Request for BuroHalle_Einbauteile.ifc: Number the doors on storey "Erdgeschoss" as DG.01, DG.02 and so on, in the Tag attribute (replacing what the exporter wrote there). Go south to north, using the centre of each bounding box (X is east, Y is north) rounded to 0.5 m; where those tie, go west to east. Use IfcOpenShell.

First a look at what the model holds.

```python
import ifcopenshell
import ifcopenshell.util.element
import ifcopenshell.util.placement

model = ifcopenshell.open("BuroHalle_Einbauteile.ifc")
print(model.schema)
storey = next(s for s in model.by_type("IfcBuildingStorey") if s.Name == "Erdgeschoss")
doors = [e for e in ifcopenshell.util.element.get_decomposition(storey) if e.is_a("IfcDoor")]
for e in sorted(doors, key=lambda e: e.id()):
    origin = ifcopenshell.util.placement.get_local_placement(e.ObjectPlacement)[:3, 3]
    print(e.id(), e.Tag, e.Name, origin.round(2) + 0.0, sep=" | ")
```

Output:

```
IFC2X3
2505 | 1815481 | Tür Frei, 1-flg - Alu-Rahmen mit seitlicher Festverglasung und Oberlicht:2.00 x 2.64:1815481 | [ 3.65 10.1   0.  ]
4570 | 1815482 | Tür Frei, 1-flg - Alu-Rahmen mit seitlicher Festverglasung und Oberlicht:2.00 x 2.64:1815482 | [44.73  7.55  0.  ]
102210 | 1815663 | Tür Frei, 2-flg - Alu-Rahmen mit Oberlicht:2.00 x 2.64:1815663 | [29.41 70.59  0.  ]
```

```python
import ifcopenshell
import ifcopenshell.geom
import ifcopenshell.util.element
import ifcopenshell.util.shape

model = ifcopenshell.open("BuroHalle_Einbauteile.ifc")
settings = ifcopenshell.geom.settings()
settings.set("use-world-coords", True)


def centre(element):
    shape = ifcopenshell.geom.create_shape(settings, element)
    return ifcopenshell.util.shape.get_bbox_centroid(shape.geometry)


storey = next(s for s in model.by_type("IfcBuildingStorey") if s.Name == "Erdgeschoss")
doors = [e for e in ifcopenshell.util.element.get_decomposition(storey) if e.is_a("IfcDoor")]

# Insertion points can sit at a corner or the storey origin, so sort by the geometry (in metres).
centres = {e: centre(e) for e in doors}
doors.sort(key=lambda e: (round(centres[e][1] / 0.5), centres[e][0]))

for i, e in enumerate(doors, start=1):
    number = f"DG.{i:02d}"
    e.Tag = number
    print(e.id(), number)

model.write("BuroHalle_Einbauteile_updated.ifc")
```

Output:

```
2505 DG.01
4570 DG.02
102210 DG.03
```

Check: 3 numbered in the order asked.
